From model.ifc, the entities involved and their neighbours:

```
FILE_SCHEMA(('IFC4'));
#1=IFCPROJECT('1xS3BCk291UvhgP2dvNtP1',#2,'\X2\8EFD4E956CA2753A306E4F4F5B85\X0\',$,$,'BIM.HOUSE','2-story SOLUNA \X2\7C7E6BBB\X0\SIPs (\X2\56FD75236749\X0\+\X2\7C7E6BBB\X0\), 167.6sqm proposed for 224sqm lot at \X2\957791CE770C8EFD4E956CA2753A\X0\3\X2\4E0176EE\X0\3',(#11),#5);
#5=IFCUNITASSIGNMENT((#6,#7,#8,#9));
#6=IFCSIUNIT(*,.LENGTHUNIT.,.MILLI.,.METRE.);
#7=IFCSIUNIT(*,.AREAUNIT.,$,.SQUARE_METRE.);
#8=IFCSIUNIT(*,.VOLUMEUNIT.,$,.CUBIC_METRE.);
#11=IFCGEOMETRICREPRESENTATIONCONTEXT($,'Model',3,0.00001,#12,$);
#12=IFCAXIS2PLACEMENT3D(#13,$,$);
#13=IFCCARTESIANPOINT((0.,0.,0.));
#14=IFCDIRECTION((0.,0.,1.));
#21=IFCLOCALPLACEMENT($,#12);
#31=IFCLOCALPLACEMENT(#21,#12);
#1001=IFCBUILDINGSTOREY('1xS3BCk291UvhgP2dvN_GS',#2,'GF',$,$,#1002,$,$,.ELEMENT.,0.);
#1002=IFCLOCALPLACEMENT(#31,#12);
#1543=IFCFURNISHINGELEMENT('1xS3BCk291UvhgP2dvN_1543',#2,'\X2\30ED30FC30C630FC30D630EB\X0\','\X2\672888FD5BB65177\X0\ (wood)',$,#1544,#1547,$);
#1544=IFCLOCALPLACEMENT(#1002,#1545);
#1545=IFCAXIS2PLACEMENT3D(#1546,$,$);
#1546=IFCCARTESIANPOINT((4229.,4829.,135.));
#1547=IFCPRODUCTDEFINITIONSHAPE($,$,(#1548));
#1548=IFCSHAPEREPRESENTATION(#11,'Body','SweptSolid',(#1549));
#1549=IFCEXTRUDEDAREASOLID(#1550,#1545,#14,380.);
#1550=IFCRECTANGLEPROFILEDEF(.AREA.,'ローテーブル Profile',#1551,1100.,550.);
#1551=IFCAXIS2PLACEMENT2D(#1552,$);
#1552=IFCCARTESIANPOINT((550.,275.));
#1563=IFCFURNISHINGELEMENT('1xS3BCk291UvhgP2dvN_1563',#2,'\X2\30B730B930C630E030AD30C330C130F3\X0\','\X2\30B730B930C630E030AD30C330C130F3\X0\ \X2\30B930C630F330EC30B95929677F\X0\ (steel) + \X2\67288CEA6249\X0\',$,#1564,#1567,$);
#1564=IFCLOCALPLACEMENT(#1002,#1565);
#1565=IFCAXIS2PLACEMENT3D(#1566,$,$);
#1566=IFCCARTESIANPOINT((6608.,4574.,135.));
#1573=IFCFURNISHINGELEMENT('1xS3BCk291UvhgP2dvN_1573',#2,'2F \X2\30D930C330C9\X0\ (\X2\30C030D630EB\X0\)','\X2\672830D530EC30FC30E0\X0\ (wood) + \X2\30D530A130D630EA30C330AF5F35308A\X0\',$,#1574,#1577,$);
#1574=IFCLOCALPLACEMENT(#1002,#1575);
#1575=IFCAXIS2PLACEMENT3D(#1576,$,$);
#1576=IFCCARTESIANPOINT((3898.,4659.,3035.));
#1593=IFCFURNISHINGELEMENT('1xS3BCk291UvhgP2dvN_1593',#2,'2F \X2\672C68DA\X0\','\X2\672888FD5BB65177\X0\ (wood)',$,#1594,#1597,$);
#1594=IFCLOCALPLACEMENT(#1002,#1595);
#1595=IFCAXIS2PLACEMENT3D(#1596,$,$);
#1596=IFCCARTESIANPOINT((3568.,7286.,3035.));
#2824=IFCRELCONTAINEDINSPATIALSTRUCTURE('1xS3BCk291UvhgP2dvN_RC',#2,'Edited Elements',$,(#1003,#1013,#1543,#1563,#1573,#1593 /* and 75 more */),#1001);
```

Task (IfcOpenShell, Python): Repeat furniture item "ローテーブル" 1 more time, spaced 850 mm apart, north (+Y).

```python
import numpy as np
import ifcopenshell
import ifcopenshell.api.geometry
import ifcopenshell.api.root
import ifcopenshell.util.element
import ifcopenshell.util.placement
import ifcopenshell.util.unit

model = ifcopenshell.open("model.ifc")
unit_scale = ifcopenshell.util.unit.calculate_unit_scale(model)


def reuse_history(source, copy):
    """copy_class also copies each property set's owner history, people and application; keep the originals."""
    for rel in copy.IsDefinedBy:
        if rel.is_a("IfcRelDefinesByProperties") and (history := rel.RelatingPropertyDefinition.OwnerHistory):
            rel.RelatingPropertyDefinition.OwnerHistory = source.OwnerHistory
            ifcopenshell.util.element.remove_deep2(model, history)


source = model.by_id(1543)
base = ifcopenshell.util.placement.get_local_placement(source.ObjectPlacement)
step = np.array([0.0, 1.0, 0.0]) * 0.85 / unit_scale

for i in range(1, 2):
    copy = ifcopenshell.api.root.copy_class(model, product=source)
    copy.Representation = ifcopenshell.util.element.copy_deep(
        model, source.Representation, exclude=["IfcGeometricRepresentationContext", "IfcRepresentationMap"]
    )
    reuse_history(source, copy)
    matrix = base.copy()
    matrix[:3, 3] += i * step
    print("added at", matrix[:3, 3].round(3) + 0.0)
    ifcopenshell.api.geometry.edit_object_placement(model, product=copy, matrix=matrix, is_si=False)

model.write("model-out.ifc")
```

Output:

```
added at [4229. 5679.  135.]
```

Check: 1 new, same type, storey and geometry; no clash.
